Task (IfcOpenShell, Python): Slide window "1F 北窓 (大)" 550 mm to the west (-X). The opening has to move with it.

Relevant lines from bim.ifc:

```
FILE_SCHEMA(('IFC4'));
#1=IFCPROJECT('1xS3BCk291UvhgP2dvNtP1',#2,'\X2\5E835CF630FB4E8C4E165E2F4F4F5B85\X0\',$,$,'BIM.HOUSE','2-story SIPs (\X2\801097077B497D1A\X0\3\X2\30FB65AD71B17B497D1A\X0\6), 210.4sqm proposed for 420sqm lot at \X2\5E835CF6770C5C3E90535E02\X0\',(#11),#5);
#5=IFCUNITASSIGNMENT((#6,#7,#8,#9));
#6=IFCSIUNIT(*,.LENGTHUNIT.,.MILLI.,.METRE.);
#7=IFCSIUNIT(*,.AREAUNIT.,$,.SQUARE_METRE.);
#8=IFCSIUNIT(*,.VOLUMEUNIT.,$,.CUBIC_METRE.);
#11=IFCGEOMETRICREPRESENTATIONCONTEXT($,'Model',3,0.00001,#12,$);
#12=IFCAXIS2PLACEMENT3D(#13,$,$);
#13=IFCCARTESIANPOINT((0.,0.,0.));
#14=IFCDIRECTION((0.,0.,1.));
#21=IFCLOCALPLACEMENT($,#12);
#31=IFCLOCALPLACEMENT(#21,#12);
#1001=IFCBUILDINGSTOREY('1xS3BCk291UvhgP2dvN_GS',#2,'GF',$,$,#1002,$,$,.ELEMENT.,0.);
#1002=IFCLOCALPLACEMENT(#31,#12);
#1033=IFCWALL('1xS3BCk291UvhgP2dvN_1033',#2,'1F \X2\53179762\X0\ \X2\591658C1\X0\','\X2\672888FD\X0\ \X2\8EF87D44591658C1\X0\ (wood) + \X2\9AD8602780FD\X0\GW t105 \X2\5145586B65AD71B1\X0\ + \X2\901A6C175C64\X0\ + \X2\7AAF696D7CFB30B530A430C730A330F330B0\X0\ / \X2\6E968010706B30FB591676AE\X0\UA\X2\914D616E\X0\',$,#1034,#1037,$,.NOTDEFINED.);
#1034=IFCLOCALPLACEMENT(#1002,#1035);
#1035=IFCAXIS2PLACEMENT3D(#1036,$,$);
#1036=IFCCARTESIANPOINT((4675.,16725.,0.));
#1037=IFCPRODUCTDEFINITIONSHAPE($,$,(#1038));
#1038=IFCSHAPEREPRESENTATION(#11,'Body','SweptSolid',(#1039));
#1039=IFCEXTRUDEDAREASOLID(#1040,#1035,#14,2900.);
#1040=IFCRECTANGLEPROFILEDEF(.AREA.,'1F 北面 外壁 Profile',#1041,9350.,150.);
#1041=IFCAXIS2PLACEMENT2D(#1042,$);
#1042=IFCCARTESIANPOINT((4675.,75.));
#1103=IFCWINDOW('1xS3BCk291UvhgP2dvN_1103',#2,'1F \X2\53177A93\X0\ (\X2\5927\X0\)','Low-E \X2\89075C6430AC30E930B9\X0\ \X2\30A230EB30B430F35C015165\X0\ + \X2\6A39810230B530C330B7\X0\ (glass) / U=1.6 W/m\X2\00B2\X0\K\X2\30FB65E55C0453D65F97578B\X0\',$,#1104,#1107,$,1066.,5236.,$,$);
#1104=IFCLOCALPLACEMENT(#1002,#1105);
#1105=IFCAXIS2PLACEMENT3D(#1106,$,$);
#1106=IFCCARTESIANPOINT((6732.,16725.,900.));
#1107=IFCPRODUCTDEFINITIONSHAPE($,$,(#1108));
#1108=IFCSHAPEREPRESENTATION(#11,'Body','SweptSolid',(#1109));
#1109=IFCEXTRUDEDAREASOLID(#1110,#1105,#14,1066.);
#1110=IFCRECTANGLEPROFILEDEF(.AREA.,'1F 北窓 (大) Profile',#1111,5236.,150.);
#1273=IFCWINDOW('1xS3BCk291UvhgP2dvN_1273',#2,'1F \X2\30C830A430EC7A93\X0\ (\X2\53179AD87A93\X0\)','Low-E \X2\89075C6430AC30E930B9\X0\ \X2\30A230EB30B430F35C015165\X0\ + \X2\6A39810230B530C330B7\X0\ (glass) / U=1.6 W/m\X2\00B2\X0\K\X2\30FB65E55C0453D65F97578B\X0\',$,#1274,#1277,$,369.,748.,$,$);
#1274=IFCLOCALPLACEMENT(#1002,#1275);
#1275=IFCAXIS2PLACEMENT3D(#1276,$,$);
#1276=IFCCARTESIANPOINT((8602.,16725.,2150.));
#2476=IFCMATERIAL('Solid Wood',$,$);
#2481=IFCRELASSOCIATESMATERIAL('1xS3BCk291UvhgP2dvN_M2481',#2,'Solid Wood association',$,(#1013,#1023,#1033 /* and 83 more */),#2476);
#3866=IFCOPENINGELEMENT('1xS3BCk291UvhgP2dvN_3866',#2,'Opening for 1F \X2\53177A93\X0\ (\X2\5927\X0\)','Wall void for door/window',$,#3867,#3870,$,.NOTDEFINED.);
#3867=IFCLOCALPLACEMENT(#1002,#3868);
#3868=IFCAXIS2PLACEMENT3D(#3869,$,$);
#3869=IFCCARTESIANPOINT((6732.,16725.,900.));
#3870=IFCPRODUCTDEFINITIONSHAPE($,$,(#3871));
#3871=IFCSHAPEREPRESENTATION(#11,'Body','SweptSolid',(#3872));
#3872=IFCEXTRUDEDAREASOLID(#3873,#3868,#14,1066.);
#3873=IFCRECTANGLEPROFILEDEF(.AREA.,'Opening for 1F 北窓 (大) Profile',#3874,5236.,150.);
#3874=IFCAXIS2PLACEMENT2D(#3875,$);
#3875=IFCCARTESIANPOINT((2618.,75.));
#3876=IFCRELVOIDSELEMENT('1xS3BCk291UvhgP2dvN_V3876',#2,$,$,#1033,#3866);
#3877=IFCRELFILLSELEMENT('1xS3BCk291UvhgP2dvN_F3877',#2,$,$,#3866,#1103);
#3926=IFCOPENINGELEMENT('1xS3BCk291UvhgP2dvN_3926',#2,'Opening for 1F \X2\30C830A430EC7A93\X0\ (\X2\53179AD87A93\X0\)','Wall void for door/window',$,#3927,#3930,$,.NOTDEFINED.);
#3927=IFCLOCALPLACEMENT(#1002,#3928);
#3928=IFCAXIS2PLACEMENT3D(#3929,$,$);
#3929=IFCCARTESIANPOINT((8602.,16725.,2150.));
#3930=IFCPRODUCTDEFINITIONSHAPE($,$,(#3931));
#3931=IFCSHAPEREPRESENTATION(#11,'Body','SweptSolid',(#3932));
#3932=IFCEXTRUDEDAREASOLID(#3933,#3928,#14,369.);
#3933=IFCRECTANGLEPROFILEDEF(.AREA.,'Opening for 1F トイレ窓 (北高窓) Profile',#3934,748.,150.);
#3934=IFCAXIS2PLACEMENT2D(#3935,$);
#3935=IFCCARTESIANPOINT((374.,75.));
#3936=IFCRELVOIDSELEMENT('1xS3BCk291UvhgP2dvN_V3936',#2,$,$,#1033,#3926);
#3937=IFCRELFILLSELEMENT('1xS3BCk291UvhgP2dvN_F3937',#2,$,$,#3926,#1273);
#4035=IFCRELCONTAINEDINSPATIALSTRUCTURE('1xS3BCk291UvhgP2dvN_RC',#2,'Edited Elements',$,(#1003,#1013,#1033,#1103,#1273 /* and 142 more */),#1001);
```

```python
import ifcopenshell
import ifcopenshell.api.geometry
import ifcopenshell.util.placement
import ifcopenshell.util.unit

model = ifcopenshell.open("bim.ifc")
unit_scale = ifcopenshell.util.unit.calculate_unit_scale(model)

window = model.by_id(1103)
opening = window.FillsVoids[0].RelatingOpeningElement
wall = opening.VoidsElements[0].RelatingBuildingElement

wall_matrix = ifcopenshell.util.placement.get_local_placement(wall.ObjectPlacement)
shift = wall_matrix[:3, 0] * -0.55 / unit_scale
before = ifcopenshell.util.placement.get_local_placement(window.ObjectPlacement)[:3, 3].copy()

# The window is not placed relative to its opening, so move both.
for product in (opening, window):
    matrix = ifcopenshell.util.placement.get_local_placement(product.ObjectPlacement)
    matrix[:3, 3] += shift
    ifcopenshell.api.geometry.edit_object_placement(model, product=product, matrix=matrix, is_si=False)

after = ifcopenshell.util.placement.get_local_placement(window.ObjectPlacement)[:3, 3]
print("window moved by", (after - before).round(3) + 0.0)

model.write("bim_v2.ifc")
```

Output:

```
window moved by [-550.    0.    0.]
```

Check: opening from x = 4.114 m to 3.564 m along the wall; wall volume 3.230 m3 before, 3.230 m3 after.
